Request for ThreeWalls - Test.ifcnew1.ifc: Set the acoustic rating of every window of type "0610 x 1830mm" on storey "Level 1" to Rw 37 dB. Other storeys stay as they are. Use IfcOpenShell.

First a look at what the model holds.

```python
import ifcopenshell
import ifcopenshell.util.element

model = ifcopenshell.open("ThreeWalls - Test.ifcnew1.ifc")
print(model.schema)
storey = next(s for s in model.by_type("IfcBuildingStorey") if s.Name == "Level 1")
windows = [e for e in ifcopenshell.util.element.get_decomposition(storey) if e.is_a("IfcWindow")]
seen = {}
for e in windows:
    element_type = ifcopenshell.util.element.get_type(e)
    key = (element_type.Name if element_type != e and element_type else None, ifcopenshell.util.element.get_pset(e, "Pset_WindowCommon", "AcousticRating"))
    seen[key] = seen.get(key, 0) + 1
for (name, value), count in sorted(seen.items(), key=str):
    print(count, "x", name, "|", value)
```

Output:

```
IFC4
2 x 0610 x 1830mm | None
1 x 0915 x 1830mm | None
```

```python
import ifcopenshell
import ifcopenshell.api.pset
import ifcopenshell.util.element

model = ifcopenshell.open("ThreeWalls - Test.ifcnew1.ifc")

storey = next(s for s in model.by_type("IfcBuildingStorey") if s.Name == "Level 1")
windows = [e for e in ifcopenshell.util.element.get_decomposition(storey) if e.is_a("IfcWindow")]

count = 0
for e in windows:
    element_type = ifcopenshell.util.element.get_type(e)
    if element_type in (None, e) or element_type.Name != "0610 x 1830mm":
        continue
    # add_pset returns the element's existing set when there is one.
    pset = ifcopenshell.api.pset.add_pset(model, product=e, name="Pset_WindowCommon")
    ifcopenshell.api.pset.edit_pset(model, pset=pset, properties={"AcousticRating": "Rw 37 dB"})
    count += 1

print(count, "windows updated")

model.write("ThreeWalls - Test.ifcnew1-out.ifc")
```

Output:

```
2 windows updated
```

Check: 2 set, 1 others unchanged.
